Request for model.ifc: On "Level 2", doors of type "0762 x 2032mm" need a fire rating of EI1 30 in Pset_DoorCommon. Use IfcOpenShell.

First a look at what the model holds.

```python
import ifcopenshell
import ifcopenshell.util.element

model = ifcopenshell.open("model.ifc")
print(model.schema)
storey = next(s for s in model.by_type("IfcBuildingStorey") if s.Name == "Level 2")
doors = [e for e in ifcopenshell.util.element.get_decomposition(storey) if e.is_a("IfcDoor")]
seen = {}
for e in doors:
    element_type = ifcopenshell.util.element.get_type(e)
    key = (element_type.Name if element_type != e and element_type else None, ifcopenshell.util.element.get_pset(e, "Pset_DoorCommon", "FireRating"))
    seen[key] = seen.get(key, 0) + 1
for (name, value), count in sorted(seen.items(), key=str):
    print(count, "x", name, "|", value)
```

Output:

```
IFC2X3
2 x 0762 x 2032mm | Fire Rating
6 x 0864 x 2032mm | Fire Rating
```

```python
import ifcopenshell
import ifcopenshell.api.pset
import ifcopenshell.util.element

model = ifcopenshell.open("model.ifc")

storey = next(s for s in model.by_type("IfcBuildingStorey") if s.Name == "Level 2")
doors = [e for e in ifcopenshell.util.element.get_decomposition(storey) if e.is_a("IfcDoor")]

count = 0
for e in doors:
    element_type = ifcopenshell.util.element.get_type(e)
    if element_type in (None, e) or element_type.Name != "0762 x 2032mm":
        continue
    # add_pset returns the element's existing set when there is one.
    pset = ifcopenshell.api.pset.add_pset(model, product=e, name="Pset_DoorCommon")
    ifcopenshell.api.pset.edit_pset(model, pset=pset, properties={"FireRating": "EI1 30"})
    count += 1

print(count, "doors updated")

model.write("model_updated.ifc")
```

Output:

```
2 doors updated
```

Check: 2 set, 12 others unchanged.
